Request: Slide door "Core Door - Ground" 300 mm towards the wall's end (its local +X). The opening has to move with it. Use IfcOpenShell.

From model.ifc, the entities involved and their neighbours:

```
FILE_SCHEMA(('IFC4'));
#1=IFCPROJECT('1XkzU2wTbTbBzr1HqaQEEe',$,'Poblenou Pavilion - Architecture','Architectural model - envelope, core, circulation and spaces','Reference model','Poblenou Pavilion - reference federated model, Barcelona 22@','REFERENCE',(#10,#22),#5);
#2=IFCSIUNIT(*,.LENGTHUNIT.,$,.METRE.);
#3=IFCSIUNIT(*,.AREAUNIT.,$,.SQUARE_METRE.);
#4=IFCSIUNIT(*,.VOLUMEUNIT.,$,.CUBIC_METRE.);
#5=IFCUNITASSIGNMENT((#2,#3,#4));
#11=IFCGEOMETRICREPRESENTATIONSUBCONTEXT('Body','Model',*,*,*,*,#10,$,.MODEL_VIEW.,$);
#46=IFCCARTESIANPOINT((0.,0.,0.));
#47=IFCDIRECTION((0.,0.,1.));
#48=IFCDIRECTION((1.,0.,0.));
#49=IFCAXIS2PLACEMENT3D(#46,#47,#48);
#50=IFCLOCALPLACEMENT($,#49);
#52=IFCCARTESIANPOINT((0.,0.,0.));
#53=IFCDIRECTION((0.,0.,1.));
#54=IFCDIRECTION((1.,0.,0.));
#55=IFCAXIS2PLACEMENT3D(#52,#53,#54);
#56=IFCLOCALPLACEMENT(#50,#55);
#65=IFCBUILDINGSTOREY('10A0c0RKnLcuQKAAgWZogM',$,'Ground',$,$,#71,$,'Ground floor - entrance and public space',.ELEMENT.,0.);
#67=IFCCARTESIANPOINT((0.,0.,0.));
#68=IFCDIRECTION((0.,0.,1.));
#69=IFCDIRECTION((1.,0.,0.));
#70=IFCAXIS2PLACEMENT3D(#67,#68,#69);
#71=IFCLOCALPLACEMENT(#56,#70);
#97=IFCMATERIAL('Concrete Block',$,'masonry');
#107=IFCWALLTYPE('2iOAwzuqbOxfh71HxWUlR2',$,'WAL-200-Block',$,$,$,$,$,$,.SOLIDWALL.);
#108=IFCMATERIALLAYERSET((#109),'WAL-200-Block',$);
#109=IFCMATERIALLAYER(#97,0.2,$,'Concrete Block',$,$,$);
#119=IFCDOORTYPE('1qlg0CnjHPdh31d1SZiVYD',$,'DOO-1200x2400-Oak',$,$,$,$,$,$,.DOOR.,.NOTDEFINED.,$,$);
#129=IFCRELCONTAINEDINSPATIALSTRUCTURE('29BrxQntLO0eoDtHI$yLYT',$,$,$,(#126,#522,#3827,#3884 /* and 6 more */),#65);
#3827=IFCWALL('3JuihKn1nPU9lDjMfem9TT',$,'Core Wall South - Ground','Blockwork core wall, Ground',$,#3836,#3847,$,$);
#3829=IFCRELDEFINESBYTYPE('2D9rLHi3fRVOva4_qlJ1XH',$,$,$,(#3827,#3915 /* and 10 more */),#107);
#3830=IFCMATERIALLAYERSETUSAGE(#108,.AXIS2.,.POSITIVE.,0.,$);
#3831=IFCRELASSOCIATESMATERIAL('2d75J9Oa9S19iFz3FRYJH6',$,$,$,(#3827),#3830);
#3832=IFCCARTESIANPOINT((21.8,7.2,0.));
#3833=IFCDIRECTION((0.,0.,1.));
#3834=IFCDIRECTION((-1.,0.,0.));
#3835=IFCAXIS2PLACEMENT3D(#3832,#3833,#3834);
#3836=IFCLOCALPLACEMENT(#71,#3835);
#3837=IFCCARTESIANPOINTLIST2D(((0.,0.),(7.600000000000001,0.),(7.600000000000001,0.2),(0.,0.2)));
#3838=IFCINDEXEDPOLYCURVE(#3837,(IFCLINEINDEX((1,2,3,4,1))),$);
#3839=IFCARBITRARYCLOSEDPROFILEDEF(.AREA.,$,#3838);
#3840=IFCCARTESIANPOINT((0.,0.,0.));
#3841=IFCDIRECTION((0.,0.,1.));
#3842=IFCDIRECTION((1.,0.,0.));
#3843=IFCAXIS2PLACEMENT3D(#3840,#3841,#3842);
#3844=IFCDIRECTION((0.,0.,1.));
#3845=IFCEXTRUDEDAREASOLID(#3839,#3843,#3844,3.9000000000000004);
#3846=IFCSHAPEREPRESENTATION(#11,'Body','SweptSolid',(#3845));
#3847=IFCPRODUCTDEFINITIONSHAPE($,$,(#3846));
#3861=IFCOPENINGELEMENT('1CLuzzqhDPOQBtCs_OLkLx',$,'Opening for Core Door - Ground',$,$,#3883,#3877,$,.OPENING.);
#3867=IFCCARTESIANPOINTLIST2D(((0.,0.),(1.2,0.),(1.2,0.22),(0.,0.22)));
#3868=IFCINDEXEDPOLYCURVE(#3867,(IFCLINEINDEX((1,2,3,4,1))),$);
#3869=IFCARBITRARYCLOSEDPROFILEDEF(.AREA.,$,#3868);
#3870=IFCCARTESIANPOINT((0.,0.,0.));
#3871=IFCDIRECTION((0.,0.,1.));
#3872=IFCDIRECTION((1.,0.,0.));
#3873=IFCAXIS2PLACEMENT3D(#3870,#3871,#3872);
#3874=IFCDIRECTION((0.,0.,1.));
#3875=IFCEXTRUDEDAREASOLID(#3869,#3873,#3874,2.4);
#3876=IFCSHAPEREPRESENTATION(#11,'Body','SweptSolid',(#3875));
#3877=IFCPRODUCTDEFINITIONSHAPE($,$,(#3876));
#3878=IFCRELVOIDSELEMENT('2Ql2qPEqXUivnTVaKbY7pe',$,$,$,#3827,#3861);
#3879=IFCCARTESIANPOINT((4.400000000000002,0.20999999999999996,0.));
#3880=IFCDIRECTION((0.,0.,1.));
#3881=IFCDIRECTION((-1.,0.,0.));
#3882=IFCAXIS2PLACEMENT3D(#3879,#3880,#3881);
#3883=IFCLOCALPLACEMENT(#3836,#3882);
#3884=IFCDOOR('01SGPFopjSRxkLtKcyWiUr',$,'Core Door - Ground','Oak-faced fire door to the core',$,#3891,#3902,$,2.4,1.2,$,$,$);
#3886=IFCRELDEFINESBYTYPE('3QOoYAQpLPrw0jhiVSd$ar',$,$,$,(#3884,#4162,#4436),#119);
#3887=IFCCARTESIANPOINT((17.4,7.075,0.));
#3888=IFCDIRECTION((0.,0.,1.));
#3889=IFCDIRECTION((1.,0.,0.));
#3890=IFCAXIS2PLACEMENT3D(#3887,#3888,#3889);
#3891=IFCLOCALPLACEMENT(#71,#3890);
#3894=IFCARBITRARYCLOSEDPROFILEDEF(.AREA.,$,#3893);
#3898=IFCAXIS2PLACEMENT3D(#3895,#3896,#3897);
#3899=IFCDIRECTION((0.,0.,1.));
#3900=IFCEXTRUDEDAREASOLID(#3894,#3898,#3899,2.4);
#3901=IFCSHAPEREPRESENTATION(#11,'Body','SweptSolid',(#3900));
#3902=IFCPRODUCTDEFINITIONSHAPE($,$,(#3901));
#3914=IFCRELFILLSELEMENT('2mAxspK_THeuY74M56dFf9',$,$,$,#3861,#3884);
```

```python
import ifcopenshell
import ifcopenshell.api.geometry
import ifcopenshell.util.placement
import ifcopenshell.util.unit

model = ifcopenshell.open("model.ifc")
unit_scale = ifcopenshell.util.unit.calculate_unit_scale(model)

door = model.by_guid("01SGPFopjSRxkLtKcyWiUr")
opening = door.FillsVoids[0].RelatingOpeningElement
wall = opening.VoidsElements[0].RelatingBuildingElement

wall_matrix = ifcopenshell.util.placement.get_local_placement(wall.ObjectPlacement)
shift = wall_matrix[:3, 0] * 0.3 / unit_scale
before = ifcopenshell.util.placement.get_local_placement(door.ObjectPlacement)[:3, 3].copy()

# The door is not placed relative to its opening, so move both.
for product in (opening, door):
    matrix = ifcopenshell.util.placement.get_local_placement(product.ObjectPlacement)
    matrix[:3, 3] += shift
    ifcopenshell.api.geometry.edit_object_placement(model, product=product, matrix=matrix, is_si=False)

after = ifcopenshell.util.placement.get_local_placement(door.ObjectPlacement)[:3, 3]
print("door moved by", (after - before).round(3) + 0.0)

model.write("model_edited.ifc")
```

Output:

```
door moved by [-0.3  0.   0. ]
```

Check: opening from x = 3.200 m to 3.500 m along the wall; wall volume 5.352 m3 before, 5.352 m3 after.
